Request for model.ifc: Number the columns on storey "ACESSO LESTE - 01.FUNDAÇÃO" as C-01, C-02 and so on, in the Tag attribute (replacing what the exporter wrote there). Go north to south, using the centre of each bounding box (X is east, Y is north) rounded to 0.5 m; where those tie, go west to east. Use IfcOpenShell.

First a look at what the model holds.

```python
import ifcopenshell
import ifcopenshell.util.element
import ifcopenshell.util.placement

model = ifcopenshell.open("model.ifc")
print(model.schema)
storey = next(s for s in model.by_type("IfcBuildingStorey") if s.Name == "ACESSO LESTE - 01.FUNDAÇÃO")
columns = [e for e in ifcopenshell.util.element.get_decomposition(storey) if e.is_a("IfcColumn")]
for e in sorted(columns, key=lambda e: e.id()):
    origin = ifcopenshell.util.placement.get_local_placement(e.ObjectPlacement)[:3, 3]
    print(e.id(), e.Tag, e.Name, origin.round(2) + 0.0, sep=" | ")
```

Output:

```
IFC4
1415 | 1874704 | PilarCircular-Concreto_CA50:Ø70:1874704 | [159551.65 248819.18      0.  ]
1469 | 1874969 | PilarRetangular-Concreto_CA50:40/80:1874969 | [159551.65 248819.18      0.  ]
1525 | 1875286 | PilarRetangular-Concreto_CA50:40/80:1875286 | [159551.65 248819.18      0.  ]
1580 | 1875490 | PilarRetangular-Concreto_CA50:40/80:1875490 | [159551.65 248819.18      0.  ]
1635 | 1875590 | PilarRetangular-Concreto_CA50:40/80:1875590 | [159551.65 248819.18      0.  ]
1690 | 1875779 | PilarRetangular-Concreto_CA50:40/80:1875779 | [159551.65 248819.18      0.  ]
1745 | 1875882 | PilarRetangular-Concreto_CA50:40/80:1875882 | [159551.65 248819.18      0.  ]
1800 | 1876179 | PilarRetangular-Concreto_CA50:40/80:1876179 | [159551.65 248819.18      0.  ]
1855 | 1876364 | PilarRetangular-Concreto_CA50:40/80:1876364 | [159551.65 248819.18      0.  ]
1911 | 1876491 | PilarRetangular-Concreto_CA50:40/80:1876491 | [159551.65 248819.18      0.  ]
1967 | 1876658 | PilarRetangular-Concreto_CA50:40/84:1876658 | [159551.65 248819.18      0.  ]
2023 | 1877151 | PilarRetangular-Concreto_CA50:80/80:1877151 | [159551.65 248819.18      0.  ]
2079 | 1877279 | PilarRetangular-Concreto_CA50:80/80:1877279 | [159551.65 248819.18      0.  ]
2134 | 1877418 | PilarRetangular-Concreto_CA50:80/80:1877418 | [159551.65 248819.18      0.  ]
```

```python
import ifcopenshell
import ifcopenshell.geom
import ifcopenshell.util.element
import ifcopenshell.util.shape

model = ifcopenshell.open("model.ifc")
settings = ifcopenshell.geom.settings()
settings.set("use-world-coords", True)


def centre(element):
    shape = ifcopenshell.geom.create_shape(settings, element)
    return ifcopenshell.util.shape.get_bbox_centroid(shape.geometry)


storey = next(s for s in model.by_type("IfcBuildingStorey") if s.Name == "ACESSO LESTE - 01.FUNDAÇÃO")
columns = [e for e in ifcopenshell.util.element.get_decomposition(storey) if e.is_a("IfcColumn")]

# Insertion points can sit at a corner or the storey origin, so sort by the geometry (in metres).
centres = {e: centre(e) for e in columns}
columns.sort(key=lambda e: (-round(centres[e][1] / 0.5), centres[e][0]))

for i, e in enumerate(columns, start=1):
    number = f"C-{i:02d}"
    e.Tag = number
    print(e.id(), number)

model.write("model_v2.ifc")
```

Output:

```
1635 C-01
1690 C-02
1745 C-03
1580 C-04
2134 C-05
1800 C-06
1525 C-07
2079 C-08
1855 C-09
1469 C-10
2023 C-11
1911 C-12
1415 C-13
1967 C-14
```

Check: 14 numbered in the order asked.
